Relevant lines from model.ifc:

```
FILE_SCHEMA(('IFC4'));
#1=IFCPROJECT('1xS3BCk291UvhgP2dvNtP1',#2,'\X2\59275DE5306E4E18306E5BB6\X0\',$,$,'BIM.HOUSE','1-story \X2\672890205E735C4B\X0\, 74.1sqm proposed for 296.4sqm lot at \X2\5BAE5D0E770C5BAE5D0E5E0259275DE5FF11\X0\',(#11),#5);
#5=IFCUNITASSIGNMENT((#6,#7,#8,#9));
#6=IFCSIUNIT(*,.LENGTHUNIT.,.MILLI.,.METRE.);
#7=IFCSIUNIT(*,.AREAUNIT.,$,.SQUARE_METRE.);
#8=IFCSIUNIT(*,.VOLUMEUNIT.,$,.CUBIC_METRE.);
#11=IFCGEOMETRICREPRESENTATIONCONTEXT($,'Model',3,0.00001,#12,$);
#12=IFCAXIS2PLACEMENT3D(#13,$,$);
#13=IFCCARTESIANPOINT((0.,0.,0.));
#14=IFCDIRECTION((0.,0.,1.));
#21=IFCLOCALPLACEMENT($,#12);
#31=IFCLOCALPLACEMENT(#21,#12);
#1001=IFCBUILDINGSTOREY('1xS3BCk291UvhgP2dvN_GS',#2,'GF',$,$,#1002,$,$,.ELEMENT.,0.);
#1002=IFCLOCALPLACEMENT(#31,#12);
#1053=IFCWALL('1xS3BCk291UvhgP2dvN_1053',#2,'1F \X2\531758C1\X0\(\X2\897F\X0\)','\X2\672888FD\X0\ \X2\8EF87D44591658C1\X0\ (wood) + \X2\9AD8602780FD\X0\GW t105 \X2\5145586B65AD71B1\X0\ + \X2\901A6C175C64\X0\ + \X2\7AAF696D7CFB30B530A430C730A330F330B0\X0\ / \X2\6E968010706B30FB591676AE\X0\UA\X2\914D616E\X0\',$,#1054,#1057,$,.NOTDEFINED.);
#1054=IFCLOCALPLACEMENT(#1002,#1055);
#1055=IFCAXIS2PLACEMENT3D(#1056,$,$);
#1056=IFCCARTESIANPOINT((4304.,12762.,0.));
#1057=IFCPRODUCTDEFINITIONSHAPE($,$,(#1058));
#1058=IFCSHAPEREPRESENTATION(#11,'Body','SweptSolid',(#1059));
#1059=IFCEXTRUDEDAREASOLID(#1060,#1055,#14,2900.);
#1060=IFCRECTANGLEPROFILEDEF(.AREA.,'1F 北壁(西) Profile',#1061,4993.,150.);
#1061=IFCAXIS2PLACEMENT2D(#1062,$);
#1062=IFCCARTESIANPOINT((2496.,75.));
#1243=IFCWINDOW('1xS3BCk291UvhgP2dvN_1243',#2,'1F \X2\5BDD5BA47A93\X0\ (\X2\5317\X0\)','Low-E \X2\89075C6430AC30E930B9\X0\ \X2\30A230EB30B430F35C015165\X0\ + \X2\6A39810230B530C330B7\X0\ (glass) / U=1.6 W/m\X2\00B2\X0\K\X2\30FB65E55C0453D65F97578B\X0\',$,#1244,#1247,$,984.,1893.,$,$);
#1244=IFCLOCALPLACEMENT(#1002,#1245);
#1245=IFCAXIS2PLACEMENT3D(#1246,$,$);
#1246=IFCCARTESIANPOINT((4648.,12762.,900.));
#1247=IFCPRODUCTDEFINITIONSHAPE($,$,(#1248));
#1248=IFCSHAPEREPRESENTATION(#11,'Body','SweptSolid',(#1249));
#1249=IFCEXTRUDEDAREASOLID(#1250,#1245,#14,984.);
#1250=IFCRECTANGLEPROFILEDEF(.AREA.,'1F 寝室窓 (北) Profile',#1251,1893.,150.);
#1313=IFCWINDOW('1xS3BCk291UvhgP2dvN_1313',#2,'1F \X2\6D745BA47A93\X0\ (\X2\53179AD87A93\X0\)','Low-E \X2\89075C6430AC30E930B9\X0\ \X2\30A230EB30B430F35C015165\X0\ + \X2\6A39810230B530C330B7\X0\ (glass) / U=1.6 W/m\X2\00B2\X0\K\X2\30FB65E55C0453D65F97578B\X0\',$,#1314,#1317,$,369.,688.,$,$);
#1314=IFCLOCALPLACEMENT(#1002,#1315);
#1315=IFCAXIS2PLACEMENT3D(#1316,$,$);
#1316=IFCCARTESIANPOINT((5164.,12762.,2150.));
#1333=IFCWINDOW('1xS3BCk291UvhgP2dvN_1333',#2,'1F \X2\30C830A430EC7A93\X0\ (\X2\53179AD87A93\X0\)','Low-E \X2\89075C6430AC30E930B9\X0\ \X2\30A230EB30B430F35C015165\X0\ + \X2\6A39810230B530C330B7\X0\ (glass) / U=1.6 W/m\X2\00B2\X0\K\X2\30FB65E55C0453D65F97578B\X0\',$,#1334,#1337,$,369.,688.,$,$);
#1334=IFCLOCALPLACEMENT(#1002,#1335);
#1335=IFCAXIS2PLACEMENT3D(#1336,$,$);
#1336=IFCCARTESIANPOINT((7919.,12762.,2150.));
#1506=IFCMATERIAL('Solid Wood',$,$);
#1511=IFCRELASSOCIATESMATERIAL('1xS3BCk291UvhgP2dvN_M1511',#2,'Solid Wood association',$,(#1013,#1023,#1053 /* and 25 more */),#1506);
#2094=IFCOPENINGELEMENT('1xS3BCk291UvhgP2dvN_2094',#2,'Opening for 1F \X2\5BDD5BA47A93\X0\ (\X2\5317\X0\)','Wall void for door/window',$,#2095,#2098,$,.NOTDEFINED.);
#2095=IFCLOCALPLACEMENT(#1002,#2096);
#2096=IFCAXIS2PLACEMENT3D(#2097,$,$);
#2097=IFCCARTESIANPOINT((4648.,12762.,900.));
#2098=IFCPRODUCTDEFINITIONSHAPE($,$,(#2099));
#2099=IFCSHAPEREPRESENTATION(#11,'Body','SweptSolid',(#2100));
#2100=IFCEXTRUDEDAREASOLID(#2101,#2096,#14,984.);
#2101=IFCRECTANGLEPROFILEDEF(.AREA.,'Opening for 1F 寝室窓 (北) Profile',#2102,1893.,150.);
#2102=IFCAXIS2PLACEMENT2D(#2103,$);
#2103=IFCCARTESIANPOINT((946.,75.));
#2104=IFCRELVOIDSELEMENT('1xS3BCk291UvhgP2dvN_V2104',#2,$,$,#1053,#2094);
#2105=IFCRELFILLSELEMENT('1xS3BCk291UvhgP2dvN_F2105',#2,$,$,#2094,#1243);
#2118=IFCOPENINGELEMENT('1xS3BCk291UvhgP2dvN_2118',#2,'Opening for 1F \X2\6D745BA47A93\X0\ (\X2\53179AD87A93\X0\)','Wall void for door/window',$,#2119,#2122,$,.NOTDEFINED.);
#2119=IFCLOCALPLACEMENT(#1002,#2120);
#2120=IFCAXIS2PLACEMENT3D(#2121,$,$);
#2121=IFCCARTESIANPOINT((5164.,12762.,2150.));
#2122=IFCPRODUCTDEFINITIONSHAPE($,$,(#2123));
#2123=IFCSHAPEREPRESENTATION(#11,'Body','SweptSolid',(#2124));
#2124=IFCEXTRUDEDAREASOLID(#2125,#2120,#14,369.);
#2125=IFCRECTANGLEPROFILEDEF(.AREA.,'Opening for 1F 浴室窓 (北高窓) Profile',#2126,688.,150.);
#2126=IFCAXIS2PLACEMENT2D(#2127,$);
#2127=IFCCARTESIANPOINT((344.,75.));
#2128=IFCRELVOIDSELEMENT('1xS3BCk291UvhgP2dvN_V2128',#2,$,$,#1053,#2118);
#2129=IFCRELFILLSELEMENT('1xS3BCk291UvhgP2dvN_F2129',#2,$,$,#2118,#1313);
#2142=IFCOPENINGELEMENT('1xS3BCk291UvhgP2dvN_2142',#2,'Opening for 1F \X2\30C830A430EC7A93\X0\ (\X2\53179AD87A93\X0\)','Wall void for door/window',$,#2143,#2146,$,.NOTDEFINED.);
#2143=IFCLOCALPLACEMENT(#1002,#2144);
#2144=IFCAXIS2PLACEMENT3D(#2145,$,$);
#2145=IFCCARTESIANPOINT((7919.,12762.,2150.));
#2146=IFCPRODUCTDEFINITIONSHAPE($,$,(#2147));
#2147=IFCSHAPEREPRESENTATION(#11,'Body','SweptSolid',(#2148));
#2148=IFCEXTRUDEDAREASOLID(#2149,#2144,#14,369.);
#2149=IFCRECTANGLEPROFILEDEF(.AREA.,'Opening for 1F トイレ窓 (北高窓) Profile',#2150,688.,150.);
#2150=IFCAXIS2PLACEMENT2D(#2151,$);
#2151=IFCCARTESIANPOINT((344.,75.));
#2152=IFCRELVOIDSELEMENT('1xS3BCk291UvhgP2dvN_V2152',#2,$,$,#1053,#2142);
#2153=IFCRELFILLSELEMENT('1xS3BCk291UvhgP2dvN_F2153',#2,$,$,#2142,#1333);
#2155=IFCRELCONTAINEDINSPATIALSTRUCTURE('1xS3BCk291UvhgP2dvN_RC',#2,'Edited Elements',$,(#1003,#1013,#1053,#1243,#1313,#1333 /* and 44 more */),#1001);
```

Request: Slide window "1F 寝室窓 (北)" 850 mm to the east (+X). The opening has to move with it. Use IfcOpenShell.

```python
import ifcopenshell
import ifcopenshell.api.geometry
import ifcopenshell.util.placement

model = ifcopenshell.open("model.ifc")

window = model.by_id(1243)
opening = window.FillsVoids[0].RelatingOpeningElement
wall = opening.VoidsElements[0].RelatingBuildingElement

wall_matrix = ifcopenshell.util.placement.get_local_placement(wall.ObjectPlacement)
shift = wall_matrix[:3, 0] * 850.0
before = ifcopenshell.util.placement.get_local_placement(window.ObjectPlacement)[:3, 3].copy()

# The window is not placed relative to its opening, so move both.
for product in (opening, window):
    matrix = ifcopenshell.util.placement.get_local_placement(product.ObjectPlacement)
    matrix[:3, 3] += shift
    ifcopenshell.api.geometry.edit_object_placement(model, product=product, matrix=matrix, is_si=False)

after = ifcopenshell.util.placement.get_local_placement(window.ObjectPlacement)[:3, 3]
print("window moved by", (after - before).round(3) + 0.0)

model.write("model_edited.ifc")
```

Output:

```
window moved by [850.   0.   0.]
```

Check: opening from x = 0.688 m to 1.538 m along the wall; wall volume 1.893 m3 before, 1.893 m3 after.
